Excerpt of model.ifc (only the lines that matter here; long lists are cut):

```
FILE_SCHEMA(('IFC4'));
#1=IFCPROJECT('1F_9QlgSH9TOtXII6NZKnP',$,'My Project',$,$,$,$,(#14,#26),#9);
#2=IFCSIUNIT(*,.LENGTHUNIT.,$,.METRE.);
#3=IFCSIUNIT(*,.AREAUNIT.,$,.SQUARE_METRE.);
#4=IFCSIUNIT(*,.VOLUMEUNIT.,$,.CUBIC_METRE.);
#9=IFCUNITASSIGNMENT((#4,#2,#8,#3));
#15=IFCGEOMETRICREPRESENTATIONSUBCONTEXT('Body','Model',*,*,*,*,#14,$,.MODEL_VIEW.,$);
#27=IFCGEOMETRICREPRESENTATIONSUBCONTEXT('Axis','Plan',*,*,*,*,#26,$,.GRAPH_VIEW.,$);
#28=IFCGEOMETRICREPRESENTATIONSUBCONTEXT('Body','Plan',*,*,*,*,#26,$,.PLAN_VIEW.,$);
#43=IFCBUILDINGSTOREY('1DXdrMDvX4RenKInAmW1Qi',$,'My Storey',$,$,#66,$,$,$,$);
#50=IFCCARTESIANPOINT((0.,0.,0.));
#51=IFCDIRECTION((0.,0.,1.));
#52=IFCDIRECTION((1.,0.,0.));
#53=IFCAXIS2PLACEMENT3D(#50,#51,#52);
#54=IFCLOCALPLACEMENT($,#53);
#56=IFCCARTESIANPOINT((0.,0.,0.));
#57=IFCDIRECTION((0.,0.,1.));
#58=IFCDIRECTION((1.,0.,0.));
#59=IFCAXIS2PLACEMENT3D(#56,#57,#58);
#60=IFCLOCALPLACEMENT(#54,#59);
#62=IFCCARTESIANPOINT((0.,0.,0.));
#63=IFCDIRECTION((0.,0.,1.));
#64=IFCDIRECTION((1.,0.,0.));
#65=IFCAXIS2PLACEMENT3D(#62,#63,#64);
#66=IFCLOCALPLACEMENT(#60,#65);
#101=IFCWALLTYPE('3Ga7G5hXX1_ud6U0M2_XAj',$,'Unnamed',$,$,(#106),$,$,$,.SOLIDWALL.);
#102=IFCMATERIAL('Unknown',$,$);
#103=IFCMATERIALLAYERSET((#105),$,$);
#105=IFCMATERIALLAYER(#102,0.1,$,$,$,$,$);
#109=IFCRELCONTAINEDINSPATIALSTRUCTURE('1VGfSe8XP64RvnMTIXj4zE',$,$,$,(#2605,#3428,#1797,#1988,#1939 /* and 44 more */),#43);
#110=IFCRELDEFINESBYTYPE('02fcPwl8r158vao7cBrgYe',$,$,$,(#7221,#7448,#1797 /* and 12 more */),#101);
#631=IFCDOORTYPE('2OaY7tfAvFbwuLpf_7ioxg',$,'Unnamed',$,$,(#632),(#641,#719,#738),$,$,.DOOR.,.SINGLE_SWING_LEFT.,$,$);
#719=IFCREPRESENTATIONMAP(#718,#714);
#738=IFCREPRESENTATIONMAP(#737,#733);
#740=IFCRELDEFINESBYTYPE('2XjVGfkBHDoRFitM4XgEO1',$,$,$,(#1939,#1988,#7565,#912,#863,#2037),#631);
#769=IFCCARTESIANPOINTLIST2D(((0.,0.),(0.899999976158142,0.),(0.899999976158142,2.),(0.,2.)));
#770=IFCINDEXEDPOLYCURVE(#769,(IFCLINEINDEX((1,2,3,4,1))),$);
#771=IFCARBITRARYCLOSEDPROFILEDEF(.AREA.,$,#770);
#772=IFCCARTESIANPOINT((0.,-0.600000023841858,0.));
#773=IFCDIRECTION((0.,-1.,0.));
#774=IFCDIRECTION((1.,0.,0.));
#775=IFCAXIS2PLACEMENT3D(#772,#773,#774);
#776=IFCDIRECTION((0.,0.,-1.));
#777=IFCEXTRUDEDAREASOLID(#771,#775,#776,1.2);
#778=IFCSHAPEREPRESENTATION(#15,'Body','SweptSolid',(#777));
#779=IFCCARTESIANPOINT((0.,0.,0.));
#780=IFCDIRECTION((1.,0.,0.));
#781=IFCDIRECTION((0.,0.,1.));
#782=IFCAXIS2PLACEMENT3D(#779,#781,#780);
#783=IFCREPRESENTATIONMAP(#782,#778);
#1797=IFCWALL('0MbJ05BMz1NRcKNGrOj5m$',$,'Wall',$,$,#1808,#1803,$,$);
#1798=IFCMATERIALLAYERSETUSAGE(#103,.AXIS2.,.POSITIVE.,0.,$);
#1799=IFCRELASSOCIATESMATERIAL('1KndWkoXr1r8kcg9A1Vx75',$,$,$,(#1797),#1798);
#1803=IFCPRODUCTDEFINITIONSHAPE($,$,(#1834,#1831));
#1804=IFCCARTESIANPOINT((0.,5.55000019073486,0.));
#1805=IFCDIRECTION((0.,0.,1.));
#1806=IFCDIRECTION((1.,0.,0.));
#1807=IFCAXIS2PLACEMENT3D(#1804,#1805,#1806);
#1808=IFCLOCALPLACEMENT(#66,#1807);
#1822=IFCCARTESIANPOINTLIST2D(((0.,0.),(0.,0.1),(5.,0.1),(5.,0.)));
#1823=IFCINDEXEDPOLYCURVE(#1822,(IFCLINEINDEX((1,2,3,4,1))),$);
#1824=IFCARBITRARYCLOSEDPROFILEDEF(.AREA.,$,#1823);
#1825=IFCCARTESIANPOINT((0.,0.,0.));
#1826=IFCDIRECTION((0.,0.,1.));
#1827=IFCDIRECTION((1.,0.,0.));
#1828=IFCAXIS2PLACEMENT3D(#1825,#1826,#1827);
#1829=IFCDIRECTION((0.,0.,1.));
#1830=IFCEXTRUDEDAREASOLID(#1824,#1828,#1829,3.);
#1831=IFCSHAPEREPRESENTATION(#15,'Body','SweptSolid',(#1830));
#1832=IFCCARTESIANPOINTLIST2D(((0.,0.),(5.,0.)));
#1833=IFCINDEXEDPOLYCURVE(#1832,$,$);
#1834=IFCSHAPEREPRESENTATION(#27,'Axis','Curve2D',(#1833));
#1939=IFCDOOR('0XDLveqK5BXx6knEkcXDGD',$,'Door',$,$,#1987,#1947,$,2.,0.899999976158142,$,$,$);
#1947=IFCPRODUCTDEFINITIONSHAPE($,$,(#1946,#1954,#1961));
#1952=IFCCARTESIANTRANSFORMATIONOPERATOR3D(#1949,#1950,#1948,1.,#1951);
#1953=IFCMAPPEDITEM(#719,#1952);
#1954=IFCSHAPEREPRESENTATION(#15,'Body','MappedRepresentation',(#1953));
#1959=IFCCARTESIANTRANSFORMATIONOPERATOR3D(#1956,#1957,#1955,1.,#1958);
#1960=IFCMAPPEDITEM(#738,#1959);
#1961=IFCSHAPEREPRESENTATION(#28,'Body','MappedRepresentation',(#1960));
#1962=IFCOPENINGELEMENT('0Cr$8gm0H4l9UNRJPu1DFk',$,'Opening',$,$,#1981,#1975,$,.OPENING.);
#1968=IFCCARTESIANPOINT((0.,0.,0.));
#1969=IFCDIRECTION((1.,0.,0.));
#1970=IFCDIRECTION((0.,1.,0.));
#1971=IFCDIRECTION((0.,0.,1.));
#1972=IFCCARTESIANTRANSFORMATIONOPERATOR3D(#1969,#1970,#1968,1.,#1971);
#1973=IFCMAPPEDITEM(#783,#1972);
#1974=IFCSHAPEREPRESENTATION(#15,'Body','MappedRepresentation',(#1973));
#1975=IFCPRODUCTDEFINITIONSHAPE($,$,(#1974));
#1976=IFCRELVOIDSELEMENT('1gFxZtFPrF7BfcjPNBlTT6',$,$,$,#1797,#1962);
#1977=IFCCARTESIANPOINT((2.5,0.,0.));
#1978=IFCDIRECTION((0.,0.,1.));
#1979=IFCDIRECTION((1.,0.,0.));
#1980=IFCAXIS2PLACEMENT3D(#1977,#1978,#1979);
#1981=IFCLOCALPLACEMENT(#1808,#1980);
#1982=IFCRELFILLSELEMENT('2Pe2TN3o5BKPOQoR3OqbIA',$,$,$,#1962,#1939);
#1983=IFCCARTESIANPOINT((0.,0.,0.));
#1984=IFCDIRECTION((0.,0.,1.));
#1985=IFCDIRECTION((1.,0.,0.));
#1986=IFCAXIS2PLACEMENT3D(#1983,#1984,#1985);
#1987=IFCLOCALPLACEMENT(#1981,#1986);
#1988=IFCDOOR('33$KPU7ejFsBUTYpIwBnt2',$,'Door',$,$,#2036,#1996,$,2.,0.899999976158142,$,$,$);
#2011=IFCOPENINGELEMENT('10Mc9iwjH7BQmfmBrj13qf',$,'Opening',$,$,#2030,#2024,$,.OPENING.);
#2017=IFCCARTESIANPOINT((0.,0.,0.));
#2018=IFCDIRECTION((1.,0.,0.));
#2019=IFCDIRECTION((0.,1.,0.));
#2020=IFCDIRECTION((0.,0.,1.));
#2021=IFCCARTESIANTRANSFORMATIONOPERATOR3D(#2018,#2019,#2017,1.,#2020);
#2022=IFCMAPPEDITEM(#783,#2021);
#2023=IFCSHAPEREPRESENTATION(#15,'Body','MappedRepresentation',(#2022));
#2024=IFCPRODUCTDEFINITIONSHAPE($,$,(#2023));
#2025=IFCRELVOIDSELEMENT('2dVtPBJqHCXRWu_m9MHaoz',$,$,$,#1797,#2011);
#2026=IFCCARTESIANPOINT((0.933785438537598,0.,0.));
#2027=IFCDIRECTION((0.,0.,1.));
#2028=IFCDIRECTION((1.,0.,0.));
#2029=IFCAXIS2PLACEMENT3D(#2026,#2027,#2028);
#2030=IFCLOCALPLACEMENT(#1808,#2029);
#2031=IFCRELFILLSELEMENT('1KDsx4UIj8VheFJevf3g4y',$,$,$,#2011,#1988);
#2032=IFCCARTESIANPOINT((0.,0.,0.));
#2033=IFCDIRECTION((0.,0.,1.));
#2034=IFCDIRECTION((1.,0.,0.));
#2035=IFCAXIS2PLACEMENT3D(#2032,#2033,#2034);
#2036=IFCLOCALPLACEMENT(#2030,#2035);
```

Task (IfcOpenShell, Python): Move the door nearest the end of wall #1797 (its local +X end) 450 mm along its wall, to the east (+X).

```python
import ifcopenshell
import ifcopenshell.api.geometry
import ifcopenshell.util.placement
import ifcopenshell.util.unit

model = ifcopenshell.open("model.ifc")
unit_scale = ifcopenshell.util.unit.calculate_unit_scale(model)

door = model.by_guid("0XDLveqK5BXx6knEkcXDGD")
opening = door.FillsVoids[0].RelatingOpeningElement
wall = opening.VoidsElements[0].RelatingBuildingElement

wall_matrix = ifcopenshell.util.placement.get_local_placement(wall.ObjectPlacement)
shift = wall_matrix[:3, 0] * 0.45 / unit_scale
before = ifcopenshell.util.placement.get_local_placement(door.ObjectPlacement)[:3, 3].copy()

# The door is placed relative to its opening, so it follows when the opening moves.
matrix = ifcopenshell.util.placement.get_local_placement(opening.ObjectPlacement)
matrix[:3, 3] += shift
ifcopenshell.api.geometry.edit_object_placement(
    model, product=opening, matrix=matrix, is_si=False, should_transform_children=True
)

after = ifcopenshell.util.placement.get_local_placement(door.ObjectPlacement)[:3, 3]
print("door moved by", (after - before).round(3) + 0.0)

model.write("model_edited.ifc")
```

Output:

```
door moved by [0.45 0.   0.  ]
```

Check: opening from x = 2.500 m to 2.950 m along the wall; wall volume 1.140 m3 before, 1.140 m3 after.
